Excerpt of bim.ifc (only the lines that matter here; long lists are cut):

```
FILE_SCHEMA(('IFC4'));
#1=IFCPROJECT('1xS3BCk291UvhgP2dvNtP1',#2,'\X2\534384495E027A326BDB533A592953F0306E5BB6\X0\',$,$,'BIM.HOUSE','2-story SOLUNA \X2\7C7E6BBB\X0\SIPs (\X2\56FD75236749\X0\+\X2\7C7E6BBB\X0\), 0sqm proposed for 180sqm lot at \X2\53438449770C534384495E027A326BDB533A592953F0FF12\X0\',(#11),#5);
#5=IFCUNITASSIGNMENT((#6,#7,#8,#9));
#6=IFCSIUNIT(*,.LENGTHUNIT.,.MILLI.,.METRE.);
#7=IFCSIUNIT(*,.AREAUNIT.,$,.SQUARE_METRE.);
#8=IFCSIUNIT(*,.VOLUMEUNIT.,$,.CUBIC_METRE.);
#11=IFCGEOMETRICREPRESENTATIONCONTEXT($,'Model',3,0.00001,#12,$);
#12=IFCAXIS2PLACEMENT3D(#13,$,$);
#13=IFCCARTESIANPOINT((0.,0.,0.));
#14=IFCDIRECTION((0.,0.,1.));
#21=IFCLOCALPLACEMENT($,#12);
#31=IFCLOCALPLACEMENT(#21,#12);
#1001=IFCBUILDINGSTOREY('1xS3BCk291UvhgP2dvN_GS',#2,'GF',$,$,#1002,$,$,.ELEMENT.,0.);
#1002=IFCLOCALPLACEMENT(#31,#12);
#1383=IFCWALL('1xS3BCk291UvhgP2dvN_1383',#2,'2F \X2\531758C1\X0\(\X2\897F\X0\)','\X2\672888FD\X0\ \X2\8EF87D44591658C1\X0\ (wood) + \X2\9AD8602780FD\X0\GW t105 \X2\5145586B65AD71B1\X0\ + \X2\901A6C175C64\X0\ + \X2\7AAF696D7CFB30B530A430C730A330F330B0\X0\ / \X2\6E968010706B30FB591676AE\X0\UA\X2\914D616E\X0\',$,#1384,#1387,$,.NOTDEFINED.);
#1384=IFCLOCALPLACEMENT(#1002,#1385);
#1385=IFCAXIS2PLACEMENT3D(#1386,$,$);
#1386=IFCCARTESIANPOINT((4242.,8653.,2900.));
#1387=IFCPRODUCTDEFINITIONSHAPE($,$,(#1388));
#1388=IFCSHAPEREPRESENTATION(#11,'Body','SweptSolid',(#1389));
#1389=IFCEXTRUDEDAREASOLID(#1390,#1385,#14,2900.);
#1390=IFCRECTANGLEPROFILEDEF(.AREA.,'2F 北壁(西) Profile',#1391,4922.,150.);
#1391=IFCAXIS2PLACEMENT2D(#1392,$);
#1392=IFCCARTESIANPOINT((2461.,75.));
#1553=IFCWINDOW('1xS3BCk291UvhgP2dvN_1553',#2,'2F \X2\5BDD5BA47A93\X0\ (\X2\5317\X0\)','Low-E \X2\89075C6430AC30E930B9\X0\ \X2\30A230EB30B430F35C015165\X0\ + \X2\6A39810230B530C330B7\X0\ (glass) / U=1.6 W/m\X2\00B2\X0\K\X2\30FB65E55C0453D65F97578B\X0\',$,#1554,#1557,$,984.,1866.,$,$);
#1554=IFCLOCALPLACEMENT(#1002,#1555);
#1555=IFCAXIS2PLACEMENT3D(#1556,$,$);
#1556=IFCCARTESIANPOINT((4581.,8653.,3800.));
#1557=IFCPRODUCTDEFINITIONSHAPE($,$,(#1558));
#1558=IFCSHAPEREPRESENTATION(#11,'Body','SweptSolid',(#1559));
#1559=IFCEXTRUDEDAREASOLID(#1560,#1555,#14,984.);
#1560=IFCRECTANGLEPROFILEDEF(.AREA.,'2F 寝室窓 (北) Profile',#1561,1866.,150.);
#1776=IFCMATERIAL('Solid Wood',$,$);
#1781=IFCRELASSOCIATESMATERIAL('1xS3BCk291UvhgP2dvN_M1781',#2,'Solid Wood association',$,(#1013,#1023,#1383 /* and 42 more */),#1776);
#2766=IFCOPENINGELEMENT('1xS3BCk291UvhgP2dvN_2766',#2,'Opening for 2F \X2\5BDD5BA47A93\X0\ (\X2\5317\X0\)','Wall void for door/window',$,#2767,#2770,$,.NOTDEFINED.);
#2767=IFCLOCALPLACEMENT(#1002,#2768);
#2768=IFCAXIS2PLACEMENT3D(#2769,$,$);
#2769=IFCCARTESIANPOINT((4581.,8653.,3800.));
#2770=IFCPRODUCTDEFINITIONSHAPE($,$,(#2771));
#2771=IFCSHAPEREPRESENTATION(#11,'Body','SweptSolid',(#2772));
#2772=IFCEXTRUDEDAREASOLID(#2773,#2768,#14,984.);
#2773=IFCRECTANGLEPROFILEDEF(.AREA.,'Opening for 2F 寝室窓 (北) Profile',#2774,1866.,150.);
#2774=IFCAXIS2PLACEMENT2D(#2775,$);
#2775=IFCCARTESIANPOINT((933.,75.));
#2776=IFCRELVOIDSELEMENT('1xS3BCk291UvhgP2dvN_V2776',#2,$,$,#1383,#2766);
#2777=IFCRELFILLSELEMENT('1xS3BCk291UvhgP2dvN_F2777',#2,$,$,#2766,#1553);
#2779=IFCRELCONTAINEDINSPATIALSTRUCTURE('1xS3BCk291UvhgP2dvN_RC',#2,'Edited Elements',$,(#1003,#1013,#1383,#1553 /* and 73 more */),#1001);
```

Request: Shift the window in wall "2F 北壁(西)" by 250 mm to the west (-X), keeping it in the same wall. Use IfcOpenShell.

```python
import ifcopenshell
import ifcopenshell.api.geometry
import ifcopenshell.util.placement
import ifcopenshell.util.unit

model = ifcopenshell.open("bim.ifc")
unit_scale = ifcopenshell.util.unit.calculate_unit_scale(model)

window = model.by_id(1553)
opening = window.FillsVoids[0].RelatingOpeningElement
wall = opening.VoidsElements[0].RelatingBuildingElement

wall_matrix = ifcopenshell.util.placement.get_local_placement(wall.ObjectPlacement)
shift = wall_matrix[:3, 0] * -0.25 / unit_scale
before = ifcopenshell.util.placement.get_local_placement(window.ObjectPlacement)[:3, 3].copy()

# The window is not placed relative to its opening, so move both.
for product in (opening, window):
    matrix = ifcopenshell.util.placement.get_local_placement(product.ObjectPlacement)
    matrix[:3, 3] += shift
    ifcopenshell.api.geometry.edit_object_placement(model, product=product, matrix=matrix, is_si=False)

after = ifcopenshell.util.placement.get_local_placement(window.ObjectPlacement)[:3, 3]
print("window moved by", (after - before).round(3) + 0.0)

model.write("bim_rev.ifc")
```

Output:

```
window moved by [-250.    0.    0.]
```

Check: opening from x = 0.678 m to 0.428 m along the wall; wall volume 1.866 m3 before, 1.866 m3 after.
